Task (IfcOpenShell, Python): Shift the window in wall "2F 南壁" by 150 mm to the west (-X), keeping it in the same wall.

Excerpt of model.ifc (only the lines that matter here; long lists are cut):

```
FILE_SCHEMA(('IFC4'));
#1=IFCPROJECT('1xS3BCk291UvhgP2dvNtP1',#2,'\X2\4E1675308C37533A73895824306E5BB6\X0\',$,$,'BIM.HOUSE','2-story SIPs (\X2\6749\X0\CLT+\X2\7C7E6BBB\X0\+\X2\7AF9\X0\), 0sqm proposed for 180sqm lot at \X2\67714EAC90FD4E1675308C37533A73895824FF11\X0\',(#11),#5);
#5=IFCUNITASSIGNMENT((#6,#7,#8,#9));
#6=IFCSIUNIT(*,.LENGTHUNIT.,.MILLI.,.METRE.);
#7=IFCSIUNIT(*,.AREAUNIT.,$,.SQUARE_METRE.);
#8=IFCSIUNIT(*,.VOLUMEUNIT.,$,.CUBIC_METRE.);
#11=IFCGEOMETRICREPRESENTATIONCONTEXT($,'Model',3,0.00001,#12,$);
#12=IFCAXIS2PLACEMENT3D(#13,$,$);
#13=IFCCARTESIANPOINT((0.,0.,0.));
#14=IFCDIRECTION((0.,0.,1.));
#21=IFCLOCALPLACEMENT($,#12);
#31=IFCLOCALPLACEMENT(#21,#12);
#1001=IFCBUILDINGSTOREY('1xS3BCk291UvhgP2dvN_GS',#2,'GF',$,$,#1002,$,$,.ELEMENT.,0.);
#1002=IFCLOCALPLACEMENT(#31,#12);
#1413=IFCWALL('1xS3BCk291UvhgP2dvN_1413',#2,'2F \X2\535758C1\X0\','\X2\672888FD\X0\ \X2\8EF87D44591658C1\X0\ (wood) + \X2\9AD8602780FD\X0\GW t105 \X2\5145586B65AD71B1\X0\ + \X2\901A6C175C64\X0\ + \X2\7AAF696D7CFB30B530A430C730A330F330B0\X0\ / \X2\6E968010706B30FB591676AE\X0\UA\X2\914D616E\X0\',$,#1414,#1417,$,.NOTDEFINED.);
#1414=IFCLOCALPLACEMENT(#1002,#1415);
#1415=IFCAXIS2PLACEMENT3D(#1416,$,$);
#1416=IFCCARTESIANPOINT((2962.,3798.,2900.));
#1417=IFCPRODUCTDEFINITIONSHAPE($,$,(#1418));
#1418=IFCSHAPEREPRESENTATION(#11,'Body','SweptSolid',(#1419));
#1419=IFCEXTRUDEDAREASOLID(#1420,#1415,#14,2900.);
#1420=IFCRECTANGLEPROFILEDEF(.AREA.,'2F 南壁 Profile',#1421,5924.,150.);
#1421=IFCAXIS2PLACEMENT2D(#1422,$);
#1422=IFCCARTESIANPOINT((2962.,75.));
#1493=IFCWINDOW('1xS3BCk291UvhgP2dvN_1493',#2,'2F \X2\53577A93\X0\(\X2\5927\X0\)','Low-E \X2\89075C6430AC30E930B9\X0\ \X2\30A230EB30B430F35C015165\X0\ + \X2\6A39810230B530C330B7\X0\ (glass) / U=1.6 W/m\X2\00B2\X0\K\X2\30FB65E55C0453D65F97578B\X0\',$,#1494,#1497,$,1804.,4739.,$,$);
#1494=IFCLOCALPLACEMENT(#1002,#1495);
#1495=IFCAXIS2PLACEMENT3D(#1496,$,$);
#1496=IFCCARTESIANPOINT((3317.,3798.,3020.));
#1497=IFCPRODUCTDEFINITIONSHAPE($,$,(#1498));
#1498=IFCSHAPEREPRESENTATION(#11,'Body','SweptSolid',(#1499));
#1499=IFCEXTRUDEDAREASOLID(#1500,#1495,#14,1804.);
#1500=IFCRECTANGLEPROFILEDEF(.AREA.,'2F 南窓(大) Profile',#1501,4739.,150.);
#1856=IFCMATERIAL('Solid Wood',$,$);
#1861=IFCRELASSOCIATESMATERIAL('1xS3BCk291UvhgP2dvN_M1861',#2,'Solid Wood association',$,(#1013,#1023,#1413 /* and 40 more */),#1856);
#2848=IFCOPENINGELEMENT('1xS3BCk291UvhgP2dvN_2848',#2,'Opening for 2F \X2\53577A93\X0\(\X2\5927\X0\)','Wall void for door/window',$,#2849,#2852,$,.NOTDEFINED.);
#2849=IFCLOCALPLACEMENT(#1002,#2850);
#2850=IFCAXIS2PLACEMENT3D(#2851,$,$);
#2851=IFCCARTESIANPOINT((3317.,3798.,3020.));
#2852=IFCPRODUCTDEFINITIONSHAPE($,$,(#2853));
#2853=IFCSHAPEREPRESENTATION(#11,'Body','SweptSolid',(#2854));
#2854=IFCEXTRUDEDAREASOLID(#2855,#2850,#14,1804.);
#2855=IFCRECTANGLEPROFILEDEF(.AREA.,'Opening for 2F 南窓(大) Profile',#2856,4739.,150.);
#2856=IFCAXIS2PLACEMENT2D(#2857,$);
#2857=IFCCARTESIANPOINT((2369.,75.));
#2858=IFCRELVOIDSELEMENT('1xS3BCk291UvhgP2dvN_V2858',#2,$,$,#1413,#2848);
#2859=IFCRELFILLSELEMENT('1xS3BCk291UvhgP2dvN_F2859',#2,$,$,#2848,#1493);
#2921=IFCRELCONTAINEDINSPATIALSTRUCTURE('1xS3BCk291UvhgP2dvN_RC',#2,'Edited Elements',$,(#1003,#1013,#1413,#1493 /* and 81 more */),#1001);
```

```python
import ifcopenshell
import ifcopenshell.api.geometry
import ifcopenshell.util.placement

model = ifcopenshell.open("model.ifc")

window = model.by_guid("1xS3BCk291UvhgP2dvN_1493")
opening = window.FillsVoids[0].RelatingOpeningElement
wall = opening.VoidsElements[0].RelatingBuildingElement

wall_matrix = ifcopenshell.util.placement.get_local_placement(wall.ObjectPlacement)
shift = wall_matrix[:3, 0] * -150.0
before = ifcopenshell.util.placement.get_local_placement(window.ObjectPlacement)[:3, 3].copy()

# The window is not placed relative to its opening, so move both.
for product in (opening, window):
    matrix = ifcopenshell.util.placement.get_local_placement(product.ObjectPlacement)
    matrix[:3, 3] += shift
    ifcopenshell.api.geometry.edit_object_placement(model, product=product, matrix=matrix, is_si=False)

after = ifcopenshell.util.placement.get_local_placement(window.ObjectPlacement)[:3, 3]
print("window moved by", (after - before).round(3) + 0.0)

model.write("model_rev.ifc")
```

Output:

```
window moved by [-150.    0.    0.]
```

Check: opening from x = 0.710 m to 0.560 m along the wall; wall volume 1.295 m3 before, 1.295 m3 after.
